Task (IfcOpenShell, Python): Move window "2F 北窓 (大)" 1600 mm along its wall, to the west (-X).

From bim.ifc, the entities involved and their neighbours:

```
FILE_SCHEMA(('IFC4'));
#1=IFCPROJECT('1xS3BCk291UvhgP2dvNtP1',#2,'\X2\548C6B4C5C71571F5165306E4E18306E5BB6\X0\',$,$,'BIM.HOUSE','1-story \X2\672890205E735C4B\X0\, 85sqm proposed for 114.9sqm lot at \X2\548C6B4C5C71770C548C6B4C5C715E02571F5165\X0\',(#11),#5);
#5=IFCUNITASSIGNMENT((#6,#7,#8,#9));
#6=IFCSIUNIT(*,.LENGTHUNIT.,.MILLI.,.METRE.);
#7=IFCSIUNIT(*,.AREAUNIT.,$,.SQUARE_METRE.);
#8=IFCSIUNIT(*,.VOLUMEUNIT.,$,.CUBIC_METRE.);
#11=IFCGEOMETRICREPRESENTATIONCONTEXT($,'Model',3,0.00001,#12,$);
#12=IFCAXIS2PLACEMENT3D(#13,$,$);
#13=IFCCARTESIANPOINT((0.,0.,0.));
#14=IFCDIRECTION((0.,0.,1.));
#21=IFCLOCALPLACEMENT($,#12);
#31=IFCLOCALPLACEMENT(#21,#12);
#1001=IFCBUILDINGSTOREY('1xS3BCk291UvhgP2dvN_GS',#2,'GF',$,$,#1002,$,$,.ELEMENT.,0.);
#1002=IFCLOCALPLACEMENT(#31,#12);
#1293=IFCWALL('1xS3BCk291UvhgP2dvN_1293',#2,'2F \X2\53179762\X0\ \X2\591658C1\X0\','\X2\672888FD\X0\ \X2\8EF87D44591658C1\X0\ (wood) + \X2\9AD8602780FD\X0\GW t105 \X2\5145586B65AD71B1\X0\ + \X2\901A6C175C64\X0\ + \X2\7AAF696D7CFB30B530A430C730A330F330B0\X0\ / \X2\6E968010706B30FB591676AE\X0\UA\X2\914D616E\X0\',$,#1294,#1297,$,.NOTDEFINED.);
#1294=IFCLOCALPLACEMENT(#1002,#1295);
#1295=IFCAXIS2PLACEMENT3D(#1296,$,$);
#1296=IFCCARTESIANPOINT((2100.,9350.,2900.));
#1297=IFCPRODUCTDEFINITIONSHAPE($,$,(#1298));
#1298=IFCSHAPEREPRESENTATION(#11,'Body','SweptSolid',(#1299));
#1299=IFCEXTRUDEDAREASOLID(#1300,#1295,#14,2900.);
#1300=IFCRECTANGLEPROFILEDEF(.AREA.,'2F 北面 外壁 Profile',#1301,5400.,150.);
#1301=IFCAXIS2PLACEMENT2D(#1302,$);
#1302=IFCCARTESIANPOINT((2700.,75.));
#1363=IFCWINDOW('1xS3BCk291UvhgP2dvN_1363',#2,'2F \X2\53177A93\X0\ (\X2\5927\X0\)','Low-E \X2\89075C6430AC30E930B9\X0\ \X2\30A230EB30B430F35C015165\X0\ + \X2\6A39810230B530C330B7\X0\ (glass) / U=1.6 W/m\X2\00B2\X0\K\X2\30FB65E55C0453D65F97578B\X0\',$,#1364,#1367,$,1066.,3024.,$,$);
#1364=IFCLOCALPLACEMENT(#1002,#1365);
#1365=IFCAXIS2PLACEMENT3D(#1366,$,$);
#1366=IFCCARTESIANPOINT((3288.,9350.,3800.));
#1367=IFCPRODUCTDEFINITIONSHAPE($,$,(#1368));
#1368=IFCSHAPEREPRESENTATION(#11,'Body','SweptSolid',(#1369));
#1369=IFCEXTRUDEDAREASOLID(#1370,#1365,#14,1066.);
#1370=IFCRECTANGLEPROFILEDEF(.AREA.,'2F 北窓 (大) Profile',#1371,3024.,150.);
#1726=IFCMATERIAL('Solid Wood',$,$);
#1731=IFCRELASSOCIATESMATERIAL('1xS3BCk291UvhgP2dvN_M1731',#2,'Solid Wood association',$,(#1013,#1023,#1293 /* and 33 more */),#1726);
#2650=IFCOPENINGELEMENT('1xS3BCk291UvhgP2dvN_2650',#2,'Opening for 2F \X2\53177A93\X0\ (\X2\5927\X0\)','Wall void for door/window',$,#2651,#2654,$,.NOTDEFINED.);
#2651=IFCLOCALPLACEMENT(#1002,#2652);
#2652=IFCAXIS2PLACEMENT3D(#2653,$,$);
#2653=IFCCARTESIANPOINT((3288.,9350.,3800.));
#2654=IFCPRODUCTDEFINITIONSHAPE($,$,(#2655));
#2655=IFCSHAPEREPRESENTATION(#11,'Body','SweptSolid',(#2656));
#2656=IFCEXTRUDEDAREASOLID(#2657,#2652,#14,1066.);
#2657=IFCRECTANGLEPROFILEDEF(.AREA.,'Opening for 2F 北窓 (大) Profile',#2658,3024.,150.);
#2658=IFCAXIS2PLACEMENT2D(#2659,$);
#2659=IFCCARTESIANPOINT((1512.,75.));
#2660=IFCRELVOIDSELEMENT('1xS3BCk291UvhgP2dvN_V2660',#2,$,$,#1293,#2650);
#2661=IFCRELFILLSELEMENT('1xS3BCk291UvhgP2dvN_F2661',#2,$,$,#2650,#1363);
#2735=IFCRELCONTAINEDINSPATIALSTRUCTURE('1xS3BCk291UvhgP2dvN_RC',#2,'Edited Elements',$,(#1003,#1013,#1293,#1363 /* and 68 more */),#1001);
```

```python
import ifcopenshell
import ifcopenshell.api.geometry
import ifcopenshell.util.placement

model = ifcopenshell.open("bim.ifc")

window = model.by_id(1363)
opening = window.FillsVoids[0].RelatingOpeningElement
wall = opening.VoidsElements[0].RelatingBuildingElement

wall_matrix = ifcopenshell.util.placement.get_local_placement(wall.ObjectPlacement)
shift = wall_matrix[:3, 0] * -1600.0
before = ifcopenshell.util.placement.get_local_placement(window.ObjectPlacement)[:3, 3].copy()

# The window is not placed relative to its opening, so move both.
for product in (opening, window):
    matrix = ifcopenshell.util.placement.get_local_placement(product.ObjectPlacement)
    matrix[:3, 3] += shift
    ifcopenshell.api.geometry.edit_object_placement(model, product=product, matrix=matrix, is_si=False)

after = ifcopenshell.util.placement.get_local_placement(window.ObjectPlacement)[:3, 3]
print("window moved by", (after - before).round(3) + 0.0)

model.write("bim_v2.ifc")
```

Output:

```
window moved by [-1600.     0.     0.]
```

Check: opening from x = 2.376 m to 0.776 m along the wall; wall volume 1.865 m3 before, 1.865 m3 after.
